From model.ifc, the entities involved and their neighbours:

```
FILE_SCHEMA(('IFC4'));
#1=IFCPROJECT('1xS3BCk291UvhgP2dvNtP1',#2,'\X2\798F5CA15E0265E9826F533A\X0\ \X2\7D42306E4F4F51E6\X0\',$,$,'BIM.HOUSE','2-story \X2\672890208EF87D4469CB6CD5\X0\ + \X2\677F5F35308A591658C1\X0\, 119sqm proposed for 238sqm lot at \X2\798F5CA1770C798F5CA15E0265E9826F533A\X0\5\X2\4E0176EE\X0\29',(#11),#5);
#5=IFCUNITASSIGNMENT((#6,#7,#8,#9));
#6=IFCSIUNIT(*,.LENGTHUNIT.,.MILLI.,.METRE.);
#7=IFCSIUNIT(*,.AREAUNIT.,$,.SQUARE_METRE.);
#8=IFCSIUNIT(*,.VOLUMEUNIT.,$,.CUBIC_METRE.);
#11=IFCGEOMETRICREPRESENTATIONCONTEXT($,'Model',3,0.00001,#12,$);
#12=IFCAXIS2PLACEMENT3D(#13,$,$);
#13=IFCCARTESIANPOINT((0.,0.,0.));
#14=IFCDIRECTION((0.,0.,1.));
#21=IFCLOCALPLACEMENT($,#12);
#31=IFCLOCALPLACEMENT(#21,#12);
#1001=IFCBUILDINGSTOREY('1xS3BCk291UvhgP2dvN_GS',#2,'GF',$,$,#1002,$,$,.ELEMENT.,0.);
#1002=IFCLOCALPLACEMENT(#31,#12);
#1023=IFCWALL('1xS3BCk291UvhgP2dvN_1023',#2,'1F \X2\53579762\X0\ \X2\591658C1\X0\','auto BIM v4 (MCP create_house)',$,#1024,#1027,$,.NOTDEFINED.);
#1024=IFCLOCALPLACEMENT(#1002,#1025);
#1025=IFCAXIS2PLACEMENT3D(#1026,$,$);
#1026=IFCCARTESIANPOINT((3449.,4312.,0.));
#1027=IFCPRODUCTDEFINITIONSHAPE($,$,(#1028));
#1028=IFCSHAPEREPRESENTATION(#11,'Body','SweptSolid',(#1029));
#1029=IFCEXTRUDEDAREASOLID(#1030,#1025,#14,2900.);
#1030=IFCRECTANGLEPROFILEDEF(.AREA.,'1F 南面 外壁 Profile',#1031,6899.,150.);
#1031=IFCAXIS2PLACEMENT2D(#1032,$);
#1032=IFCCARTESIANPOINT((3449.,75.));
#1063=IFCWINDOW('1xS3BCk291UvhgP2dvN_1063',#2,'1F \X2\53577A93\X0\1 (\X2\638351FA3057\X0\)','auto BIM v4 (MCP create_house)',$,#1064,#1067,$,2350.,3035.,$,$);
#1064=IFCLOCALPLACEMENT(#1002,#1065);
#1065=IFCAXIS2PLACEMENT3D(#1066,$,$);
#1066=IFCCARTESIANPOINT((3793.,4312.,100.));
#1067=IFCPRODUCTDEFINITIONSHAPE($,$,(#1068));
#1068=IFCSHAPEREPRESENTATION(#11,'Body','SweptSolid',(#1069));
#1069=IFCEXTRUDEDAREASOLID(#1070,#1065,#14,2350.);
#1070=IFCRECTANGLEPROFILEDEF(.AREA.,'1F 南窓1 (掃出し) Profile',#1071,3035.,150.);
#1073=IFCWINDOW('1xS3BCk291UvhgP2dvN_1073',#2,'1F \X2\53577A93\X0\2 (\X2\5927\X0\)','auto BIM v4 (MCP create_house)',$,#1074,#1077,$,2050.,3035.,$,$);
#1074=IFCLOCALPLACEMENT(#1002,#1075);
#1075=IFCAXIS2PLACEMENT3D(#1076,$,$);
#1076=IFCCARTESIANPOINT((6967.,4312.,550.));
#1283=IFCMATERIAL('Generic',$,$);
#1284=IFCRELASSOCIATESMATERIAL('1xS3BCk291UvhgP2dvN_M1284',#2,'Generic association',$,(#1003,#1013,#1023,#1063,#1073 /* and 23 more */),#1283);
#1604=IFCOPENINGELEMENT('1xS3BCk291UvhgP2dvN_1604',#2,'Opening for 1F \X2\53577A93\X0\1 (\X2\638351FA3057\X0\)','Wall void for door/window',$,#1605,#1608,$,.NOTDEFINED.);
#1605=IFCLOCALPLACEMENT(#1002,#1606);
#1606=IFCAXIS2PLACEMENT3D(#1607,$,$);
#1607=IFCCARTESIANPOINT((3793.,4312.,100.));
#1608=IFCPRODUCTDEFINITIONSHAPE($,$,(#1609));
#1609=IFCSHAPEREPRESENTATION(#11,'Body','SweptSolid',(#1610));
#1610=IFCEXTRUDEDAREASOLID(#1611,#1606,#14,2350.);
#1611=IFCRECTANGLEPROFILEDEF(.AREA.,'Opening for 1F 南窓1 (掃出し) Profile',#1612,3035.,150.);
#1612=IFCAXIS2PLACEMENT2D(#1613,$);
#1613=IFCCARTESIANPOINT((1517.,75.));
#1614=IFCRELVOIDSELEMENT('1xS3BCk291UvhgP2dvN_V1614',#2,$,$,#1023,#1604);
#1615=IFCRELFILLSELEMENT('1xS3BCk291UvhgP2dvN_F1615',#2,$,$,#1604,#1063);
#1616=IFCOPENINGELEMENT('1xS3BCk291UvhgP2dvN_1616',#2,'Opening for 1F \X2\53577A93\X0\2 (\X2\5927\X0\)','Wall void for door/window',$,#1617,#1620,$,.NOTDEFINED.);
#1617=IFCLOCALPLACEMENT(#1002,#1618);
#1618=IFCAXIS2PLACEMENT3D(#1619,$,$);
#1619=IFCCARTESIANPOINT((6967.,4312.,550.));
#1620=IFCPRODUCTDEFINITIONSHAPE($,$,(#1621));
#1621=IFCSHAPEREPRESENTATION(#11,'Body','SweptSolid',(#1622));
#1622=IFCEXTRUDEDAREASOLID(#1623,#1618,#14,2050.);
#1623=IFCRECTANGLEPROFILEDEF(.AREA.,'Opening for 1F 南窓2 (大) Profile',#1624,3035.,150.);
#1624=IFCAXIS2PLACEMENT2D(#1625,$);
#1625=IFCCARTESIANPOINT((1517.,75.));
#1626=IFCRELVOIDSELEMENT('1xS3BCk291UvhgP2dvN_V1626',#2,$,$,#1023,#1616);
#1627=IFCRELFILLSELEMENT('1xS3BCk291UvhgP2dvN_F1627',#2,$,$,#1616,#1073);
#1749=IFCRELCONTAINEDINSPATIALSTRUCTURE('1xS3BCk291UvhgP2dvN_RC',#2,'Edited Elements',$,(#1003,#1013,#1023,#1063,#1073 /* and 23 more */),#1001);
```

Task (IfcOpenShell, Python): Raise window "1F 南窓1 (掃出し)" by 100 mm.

```python
import numpy as np
import ifcopenshell
import ifcopenshell.api.geometry
import ifcopenshell.util.placement
import ifcopenshell.util.unit

model = ifcopenshell.open("model.ifc")
unit_scale = ifcopenshell.util.unit.calculate_unit_scale(model)

window = model.by_id(1063)
opening = window.FillsVoids[0].RelatingOpeningElement
dz = 0.1 / unit_scale

shift = np.array([0.0, 0.0, dz])
# The window is not placed relative to its opening, so move both.
for product in (opening, window):
    matrix = ifcopenshell.util.placement.get_local_placement(product.ObjectPlacement)
    matrix[:3, 3] += shift
    ifcopenshell.api.geometry.edit_object_placement(model, product=product, matrix=matrix, is_si=False)

print(f"moved by {dz * unit_scale:+.3f} m")

model.write("model_edited.ifc")
```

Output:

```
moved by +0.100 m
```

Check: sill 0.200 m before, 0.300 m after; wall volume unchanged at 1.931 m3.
